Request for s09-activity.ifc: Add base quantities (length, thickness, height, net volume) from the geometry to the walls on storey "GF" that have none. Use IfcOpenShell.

First a look at what the model holds.

```python
import ifcopenshell
import ifcopenshell.util.element
import ifcopenshell.util.unit

model = ifcopenshell.open("s09-activity.ifc")
print(model.schema)
for unit_type in ("LENGTHUNIT", "AREAUNIT", "VOLUMEUNIT"):
    print(unit_type, ifcopenshell.util.unit.calculate_unit_scale(model, unit_type))
storey = next(s for s in model.by_type("IfcBuildingStorey") if s.Name == "GF")
walls = [e for e in ifcopenshell.util.element.get_decomposition(storey) if e.is_a("IfcWall")]
for e in sorted(walls, key=lambda e: e.id()):
    print(e.id(), e.is_a(), e.Name, list(ifcopenshell.util.element.get_psets(e, qtos_only=True)), sep=" | ")
```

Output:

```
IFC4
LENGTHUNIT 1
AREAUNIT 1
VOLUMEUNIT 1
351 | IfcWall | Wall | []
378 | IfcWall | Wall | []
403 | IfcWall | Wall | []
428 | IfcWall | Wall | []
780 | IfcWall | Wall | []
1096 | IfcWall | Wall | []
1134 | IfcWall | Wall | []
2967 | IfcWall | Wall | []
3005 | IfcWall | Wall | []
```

```python
import ifcopenshell
import ifcopenshell.api.pset
import ifcopenshell.geom
import ifcopenshell.util.element
import ifcopenshell.util.shape
import ifcopenshell.util.unit

model = ifcopenshell.open("s09-activity.ifc")
unit_scale = ifcopenshell.util.unit.calculate_unit_scale(model)
volume_scale = ifcopenshell.util.unit.calculate_unit_scale(model, "VOLUMEUNIT")
settings = ifcopenshell.geom.settings()

storey = next(s for s in model.by_type("IfcBuildingStorey") if s.Name == "GF")
walls = [e for e in ifcopenshell.util.element.get_decomposition(storey) if e.is_a("IfcWall")]

for e in sorted(walls, key=lambda e: e.id()):
    if ifcopenshell.util.element.get_psets(e, qtos_only=True, should_inherit=False):
        continue
    # Geometry comes back in metres, in the element's own axes.
    shape = ifcopenshell.geom.create_shape(settings, e)
    values = {
        "Length": ifcopenshell.util.shape.get_x(shape.geometry) / unit_scale,
        "Width": ifcopenshell.util.shape.get_y(shape.geometry) / unit_scale,
        "Height": ifcopenshell.util.shape.get_z(shape.geometry) / unit_scale,
        "NetVolume": ifcopenshell.util.shape.get_volume(shape.geometry) / volume_scale,
    }
    qto = ifcopenshell.api.pset.add_qto(model, product=e, name="Qto_WallBaseQuantities")
    ifcopenshell.api.pset.edit_qto(model, qto=qto, properties=values)
    print(e.id(), {k: round(v, 3) for k, v in values.items()})

model.write("s09-activity_edited.ifc")
```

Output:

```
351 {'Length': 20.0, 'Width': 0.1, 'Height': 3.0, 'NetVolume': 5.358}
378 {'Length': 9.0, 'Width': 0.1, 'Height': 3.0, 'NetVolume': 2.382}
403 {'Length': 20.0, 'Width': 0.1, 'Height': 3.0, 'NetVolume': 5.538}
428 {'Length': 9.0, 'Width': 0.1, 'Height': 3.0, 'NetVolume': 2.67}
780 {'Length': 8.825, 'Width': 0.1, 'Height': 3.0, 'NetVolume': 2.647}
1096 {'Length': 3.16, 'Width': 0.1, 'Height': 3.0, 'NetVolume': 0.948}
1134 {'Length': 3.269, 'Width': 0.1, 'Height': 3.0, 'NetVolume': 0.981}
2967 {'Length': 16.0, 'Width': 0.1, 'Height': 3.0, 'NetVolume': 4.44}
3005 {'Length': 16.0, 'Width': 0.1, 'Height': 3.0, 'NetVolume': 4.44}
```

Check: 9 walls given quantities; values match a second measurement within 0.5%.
